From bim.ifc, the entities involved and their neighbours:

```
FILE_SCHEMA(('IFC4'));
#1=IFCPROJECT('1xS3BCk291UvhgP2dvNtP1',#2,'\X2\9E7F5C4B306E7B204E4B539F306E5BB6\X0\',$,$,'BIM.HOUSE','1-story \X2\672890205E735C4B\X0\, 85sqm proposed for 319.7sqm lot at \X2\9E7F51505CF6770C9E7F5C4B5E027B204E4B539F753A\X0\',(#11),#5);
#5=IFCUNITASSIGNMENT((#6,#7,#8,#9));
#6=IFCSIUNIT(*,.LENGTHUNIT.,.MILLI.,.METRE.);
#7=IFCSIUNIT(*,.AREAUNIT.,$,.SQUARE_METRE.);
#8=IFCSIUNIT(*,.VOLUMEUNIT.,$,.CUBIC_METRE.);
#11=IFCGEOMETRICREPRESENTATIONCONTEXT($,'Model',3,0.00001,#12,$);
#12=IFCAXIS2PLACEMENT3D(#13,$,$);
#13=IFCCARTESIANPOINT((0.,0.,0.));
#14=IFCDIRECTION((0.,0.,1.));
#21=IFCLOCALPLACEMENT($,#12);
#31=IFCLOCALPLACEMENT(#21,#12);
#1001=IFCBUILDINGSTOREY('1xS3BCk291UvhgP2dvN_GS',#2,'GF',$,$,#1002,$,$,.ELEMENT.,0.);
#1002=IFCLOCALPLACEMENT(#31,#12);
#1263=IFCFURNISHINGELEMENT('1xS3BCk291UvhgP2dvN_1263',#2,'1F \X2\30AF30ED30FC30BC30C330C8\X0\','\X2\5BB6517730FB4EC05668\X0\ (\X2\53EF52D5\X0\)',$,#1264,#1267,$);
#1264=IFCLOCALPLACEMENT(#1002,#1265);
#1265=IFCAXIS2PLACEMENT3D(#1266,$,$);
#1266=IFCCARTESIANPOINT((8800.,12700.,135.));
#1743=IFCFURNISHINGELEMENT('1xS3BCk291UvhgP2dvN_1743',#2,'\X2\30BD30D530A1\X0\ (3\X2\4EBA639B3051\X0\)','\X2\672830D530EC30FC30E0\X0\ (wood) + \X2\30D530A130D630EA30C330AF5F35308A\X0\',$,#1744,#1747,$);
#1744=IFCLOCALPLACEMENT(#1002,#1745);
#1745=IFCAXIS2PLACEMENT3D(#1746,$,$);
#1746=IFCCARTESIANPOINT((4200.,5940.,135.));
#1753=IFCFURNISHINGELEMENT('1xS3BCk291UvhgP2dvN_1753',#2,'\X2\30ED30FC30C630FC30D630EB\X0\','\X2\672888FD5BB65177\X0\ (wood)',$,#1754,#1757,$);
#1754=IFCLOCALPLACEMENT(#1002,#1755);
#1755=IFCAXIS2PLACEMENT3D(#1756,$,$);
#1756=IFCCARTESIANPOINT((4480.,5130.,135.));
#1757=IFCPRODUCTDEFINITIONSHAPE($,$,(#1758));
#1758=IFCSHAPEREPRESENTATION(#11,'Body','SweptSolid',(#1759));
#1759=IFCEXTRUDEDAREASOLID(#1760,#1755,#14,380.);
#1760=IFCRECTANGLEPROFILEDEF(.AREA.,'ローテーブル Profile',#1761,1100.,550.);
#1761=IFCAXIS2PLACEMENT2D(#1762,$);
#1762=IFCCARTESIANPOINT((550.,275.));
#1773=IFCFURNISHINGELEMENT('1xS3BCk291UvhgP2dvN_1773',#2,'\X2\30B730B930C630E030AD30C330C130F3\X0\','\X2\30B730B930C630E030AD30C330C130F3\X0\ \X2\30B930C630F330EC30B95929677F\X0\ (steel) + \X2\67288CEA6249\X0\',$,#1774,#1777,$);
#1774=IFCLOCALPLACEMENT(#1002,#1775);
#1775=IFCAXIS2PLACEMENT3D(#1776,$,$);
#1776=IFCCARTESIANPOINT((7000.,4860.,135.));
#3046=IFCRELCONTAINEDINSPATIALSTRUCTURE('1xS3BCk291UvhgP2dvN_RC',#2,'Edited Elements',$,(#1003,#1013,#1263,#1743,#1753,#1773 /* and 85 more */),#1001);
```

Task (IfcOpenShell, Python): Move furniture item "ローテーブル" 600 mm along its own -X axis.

```python
import ifcopenshell
import ifcopenshell.api.geometry
import ifcopenshell.util.placement

model = ifcopenshell.open("bim.ifc")

item = model.by_guid("1xS3BCk291UvhgP2dvN_1753")
matrix = ifcopenshell.util.placement.get_local_placement(item.ObjectPlacement)
matrix[:3, 3] -= matrix[:3, 0] * 600.0
ifcopenshell.api.geometry.edit_object_placement(model, product=item, matrix=matrix, is_si=False)

print(ifcopenshell.util.placement.get_local_placement(item.ObjectPlacement).round(3) + 0.0)

model.write("bim_updated.ifc")
```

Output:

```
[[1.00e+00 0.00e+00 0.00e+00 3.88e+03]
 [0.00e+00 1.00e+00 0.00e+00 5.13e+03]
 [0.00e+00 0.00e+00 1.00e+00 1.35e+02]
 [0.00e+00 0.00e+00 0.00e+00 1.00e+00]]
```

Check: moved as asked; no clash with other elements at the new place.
